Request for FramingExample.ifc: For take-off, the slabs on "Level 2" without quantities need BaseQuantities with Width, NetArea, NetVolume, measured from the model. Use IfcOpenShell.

First a look at what the model holds.

```python
import ifcopenshell
import ifcopenshell.util.element
import ifcopenshell.util.unit

model = ifcopenshell.open("FramingExample.ifc")
print(model.schema)
for unit_type in ("LENGTHUNIT", "AREAUNIT", "VOLUMEUNIT"):
    print(unit_type, ifcopenshell.util.unit.calculate_unit_scale(model, unit_type))
storey = next(s for s in model.by_type("IfcBuildingStorey") if s.Name == "Level 2")
slabs = [e for e in ifcopenshell.util.element.get_decomposition(storey) if e.is_a("IfcSlab")]
for e in sorted(slabs, key=lambda e: e.id()):
    print(e.id(), e.is_a(), e.Name, list(ifcopenshell.util.element.get_psets(e, qtos_only=True)), sep=" | ")
```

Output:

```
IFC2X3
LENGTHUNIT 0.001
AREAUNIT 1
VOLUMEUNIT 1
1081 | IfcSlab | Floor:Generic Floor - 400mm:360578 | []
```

```python
import ifcopenshell
import ifcopenshell.api.pset
import ifcopenshell.geom
import ifcopenshell.util.element
import ifcopenshell.util.shape
import ifcopenshell.util.unit

model = ifcopenshell.open("FramingExample.ifc")
unit_scale = ifcopenshell.util.unit.calculate_unit_scale(model)
area_scale = ifcopenshell.util.unit.calculate_unit_scale(model, "AREAUNIT")
volume_scale = ifcopenshell.util.unit.calculate_unit_scale(model, "VOLUMEUNIT")
settings = ifcopenshell.geom.settings()

storey = next(s for s in model.by_type("IfcBuildingStorey") if s.Name == "Level 2")
slabs = [e for e in ifcopenshell.util.element.get_decomposition(storey) if e.is_a("IfcSlab")]

for e in sorted(slabs, key=lambda e: e.id()):
    if ifcopenshell.util.element.get_psets(e, qtos_only=True, should_inherit=False):
        continue
    # Geometry comes back in metres, in the element's own axes.
    shape = ifcopenshell.geom.create_shape(settings, e)
    values = {
        "Width": ifcopenshell.util.shape.get_z(shape.geometry) / unit_scale,
        "NetArea": ifcopenshell.util.shape.get_footprint_area(shape.geometry) / area_scale,
        "NetVolume": ifcopenshell.util.shape.get_volume(shape.geometry) / volume_scale,
    }
    qto = ifcopenshell.api.pset.add_qto(model, product=e, name="BaseQuantities")
    ifcopenshell.api.pset.edit_qto(model, qto=qto, properties=values)
    print(e.id(), {k: round(v, 3) for k, v in values.items()})

model.write("FramingExample_v2.ifc")
```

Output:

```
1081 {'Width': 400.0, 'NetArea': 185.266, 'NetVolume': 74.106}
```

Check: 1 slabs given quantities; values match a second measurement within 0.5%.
